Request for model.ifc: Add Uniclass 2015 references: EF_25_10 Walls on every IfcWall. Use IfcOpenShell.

First a look at what the model holds.

```python
import ifcopenshell

model = ifcopenshell.open("model.ifc")
print(model.schema)
print("classifications:", [c.Name for c in model.by_type("IfcClassification")])
for ifc_class in ("IfcDoor", "IfcRoof", "IfcStair", "IfcWall", "IfcWindow"):
    print(ifc_class, len(model.by_type(ifc_class)))
```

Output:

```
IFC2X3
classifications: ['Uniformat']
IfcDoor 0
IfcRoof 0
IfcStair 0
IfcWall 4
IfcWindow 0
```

```python
import ifcopenshell
import ifcopenshell.api.classification

model = ifcopenshell.open("model.ifc")

# IFC2X3 requires Source and Edition and has no link from the project to the system.
system = model.create_entity("IfcClassification", Source="NBS", Edition="2015", Name="Uniclass 2015")

codes = {
    "IfcWall": ("EF_25_10", "Walls"),
}
for ifc_class, (code, name) in codes.items():
    products = model.by_type(ifc_class)
    ifcopenshell.api.classification.add_reference(
        model, products=products, classification=system, identification=code, name=name
    )
    print(code, len(products))

model.write("model-out.ifc")
```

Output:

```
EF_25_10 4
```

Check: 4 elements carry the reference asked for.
